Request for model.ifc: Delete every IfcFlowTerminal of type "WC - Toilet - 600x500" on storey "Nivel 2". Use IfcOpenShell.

First a look at what the model holds.

```python
import ifcopenshell
import ifcopenshell.util.element

model = ifcopenshell.open("model.ifc")
print(model.schema)
storey = next(s for s in model.by_type("IfcBuildingStorey") if s.Name == "Nivel 2")
terminals = [e for e in ifcopenshell.util.element.get_decomposition(storey) if e.is_a("IfcFlowTerminal")]
seen = {}
for e in terminals:
    element_type = ifcopenshell.util.element.get_type(e)
    name = element_type.Name if element_type not in (None, e) else None
    seen[name] = seen.get(name, 0) + 1
for name, count in sorted(seen.items(), key=str):
    print(count, "x", name)
```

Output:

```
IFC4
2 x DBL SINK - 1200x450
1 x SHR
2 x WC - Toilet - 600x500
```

```python
import ifcopenshell
import ifcopenshell.api.root
import ifcopenshell.util.element

model = ifcopenshell.open("model.ifc")

storey = next(s for s in model.by_type("IfcBuildingStorey") if s.Name == "Nivel 2")
terminals = [e for e in ifcopenshell.util.element.get_decomposition(storey) if e.is_a("IfcFlowTerminal")]
targets = [e for e in terminals if (t := ifcopenshell.util.element.get_type(e)) not in (None, e) and t.Name == "WC - Toilet - 600x500"]

for e in targets:
    ifcopenshell.api.root.remove_product(model, product=e)
print(len(targets), "removed")

model.write("model_rev.ifc")
```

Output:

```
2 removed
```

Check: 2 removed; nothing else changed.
